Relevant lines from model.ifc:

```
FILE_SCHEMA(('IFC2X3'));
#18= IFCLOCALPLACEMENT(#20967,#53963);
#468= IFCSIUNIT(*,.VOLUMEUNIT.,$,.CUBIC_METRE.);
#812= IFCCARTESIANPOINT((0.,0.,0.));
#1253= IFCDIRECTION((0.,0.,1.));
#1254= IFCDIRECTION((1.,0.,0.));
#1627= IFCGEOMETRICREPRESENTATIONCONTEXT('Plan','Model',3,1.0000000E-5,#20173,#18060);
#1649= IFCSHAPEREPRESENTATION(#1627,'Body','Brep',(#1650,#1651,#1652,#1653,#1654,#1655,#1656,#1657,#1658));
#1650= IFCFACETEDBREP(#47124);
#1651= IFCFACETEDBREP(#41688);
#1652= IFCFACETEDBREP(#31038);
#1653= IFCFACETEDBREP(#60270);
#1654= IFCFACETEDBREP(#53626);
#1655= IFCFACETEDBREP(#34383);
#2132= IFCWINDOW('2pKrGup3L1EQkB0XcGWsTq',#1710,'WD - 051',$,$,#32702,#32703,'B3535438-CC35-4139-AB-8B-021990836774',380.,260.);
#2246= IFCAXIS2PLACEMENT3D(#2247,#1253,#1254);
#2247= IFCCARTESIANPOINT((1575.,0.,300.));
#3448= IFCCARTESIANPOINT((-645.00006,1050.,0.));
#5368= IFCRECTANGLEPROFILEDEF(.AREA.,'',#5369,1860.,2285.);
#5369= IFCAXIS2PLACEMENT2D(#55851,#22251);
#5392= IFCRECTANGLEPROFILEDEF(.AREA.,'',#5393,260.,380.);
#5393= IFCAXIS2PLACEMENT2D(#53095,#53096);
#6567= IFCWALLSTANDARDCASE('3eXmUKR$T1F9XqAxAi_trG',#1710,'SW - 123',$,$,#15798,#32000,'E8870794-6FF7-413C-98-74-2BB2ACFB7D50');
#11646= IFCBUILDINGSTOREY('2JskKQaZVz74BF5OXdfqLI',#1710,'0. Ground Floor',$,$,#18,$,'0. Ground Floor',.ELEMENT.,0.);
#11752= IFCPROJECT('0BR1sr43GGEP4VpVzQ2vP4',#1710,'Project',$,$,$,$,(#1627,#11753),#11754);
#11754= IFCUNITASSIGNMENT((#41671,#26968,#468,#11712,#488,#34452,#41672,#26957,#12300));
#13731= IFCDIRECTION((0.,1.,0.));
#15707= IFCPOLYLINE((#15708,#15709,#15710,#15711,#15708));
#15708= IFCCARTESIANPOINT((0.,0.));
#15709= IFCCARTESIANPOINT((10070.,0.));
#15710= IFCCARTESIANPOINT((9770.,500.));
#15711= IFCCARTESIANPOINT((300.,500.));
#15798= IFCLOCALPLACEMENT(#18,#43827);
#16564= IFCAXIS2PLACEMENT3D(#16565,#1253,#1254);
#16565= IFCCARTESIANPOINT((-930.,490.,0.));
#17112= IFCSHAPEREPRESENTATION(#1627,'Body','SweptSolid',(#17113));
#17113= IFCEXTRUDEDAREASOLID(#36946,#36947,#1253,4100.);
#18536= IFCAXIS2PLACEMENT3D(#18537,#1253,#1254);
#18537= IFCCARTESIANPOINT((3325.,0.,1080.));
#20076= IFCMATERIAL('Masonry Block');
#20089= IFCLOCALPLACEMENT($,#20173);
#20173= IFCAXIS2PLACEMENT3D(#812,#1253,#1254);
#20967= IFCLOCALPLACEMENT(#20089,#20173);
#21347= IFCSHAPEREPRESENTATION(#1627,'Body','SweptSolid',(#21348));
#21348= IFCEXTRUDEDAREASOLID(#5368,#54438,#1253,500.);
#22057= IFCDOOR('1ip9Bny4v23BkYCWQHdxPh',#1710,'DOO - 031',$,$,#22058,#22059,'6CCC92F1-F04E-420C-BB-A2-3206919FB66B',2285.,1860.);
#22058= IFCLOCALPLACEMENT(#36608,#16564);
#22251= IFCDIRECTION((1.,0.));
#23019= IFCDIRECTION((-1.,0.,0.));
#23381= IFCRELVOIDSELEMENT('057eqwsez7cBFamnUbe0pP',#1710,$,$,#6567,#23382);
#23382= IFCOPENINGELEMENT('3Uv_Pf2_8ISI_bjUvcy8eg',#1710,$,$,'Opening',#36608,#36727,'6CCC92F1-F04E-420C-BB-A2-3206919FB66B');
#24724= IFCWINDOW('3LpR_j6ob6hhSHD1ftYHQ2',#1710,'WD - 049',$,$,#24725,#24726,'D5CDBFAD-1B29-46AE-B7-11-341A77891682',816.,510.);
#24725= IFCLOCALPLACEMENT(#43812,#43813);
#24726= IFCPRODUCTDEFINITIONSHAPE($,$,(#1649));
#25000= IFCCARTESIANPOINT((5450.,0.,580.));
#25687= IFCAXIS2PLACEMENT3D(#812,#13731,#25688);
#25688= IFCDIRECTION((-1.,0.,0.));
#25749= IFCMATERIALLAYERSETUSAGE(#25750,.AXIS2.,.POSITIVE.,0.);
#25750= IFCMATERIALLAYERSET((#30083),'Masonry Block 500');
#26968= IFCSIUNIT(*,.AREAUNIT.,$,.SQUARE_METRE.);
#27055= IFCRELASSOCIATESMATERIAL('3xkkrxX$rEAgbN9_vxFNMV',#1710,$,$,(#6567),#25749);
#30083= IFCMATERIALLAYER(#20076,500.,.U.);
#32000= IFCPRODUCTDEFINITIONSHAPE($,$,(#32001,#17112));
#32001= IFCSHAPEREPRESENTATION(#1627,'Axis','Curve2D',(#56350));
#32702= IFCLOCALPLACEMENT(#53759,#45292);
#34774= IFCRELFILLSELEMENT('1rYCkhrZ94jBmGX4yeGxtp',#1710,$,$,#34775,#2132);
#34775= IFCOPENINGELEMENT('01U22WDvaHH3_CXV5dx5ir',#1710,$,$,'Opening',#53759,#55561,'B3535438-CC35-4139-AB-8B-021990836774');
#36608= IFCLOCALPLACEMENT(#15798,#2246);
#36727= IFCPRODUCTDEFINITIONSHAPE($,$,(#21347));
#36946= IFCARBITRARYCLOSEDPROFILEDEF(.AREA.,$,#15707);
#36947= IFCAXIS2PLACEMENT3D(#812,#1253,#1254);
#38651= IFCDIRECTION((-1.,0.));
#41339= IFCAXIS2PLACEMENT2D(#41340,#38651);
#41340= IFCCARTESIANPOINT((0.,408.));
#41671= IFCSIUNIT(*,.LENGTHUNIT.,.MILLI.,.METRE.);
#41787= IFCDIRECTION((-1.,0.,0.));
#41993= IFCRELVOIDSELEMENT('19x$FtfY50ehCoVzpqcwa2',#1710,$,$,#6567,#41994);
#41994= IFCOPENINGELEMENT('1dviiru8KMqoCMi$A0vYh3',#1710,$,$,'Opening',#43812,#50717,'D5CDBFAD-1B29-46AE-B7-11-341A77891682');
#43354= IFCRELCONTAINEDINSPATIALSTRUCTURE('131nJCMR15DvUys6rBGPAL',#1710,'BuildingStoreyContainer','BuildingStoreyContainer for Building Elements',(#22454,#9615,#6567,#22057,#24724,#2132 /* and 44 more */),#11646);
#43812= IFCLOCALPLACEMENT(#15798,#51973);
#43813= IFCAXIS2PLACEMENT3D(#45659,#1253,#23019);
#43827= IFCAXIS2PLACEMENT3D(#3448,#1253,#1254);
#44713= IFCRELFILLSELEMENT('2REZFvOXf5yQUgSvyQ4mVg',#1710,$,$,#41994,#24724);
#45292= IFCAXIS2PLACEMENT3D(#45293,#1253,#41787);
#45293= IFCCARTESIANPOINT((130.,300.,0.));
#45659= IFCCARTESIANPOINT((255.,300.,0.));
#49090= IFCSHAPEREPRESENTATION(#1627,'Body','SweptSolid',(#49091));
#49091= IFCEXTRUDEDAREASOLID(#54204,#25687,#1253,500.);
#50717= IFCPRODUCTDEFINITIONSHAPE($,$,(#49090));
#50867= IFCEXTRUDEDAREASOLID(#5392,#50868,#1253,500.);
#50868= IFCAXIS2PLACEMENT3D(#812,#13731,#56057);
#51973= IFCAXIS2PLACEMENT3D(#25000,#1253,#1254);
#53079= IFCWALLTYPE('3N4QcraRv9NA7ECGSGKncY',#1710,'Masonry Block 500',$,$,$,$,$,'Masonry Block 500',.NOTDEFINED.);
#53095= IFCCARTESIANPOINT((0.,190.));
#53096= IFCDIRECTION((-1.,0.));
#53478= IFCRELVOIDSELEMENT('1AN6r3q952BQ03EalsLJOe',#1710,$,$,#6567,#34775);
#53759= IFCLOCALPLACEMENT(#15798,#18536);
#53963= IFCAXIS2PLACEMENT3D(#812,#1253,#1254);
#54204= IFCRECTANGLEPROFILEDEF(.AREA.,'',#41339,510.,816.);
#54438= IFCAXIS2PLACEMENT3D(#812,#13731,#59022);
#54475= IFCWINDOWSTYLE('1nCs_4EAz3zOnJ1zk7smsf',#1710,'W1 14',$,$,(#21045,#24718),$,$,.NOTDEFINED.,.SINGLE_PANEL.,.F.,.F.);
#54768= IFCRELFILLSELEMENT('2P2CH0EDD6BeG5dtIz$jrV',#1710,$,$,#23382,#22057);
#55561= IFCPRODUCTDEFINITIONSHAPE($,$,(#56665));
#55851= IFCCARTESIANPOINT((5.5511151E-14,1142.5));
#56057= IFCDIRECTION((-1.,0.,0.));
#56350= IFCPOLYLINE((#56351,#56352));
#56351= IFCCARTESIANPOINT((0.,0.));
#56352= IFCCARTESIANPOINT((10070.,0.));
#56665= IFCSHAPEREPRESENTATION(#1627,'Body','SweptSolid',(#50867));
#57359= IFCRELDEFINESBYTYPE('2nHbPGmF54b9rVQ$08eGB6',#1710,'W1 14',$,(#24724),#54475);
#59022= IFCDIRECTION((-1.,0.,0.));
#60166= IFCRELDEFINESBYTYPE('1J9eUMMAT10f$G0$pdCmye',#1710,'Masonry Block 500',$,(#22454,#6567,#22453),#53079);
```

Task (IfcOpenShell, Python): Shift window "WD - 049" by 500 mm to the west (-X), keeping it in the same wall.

```python
import ifcopenshell
import ifcopenshell.api.geometry
import ifcopenshell.util.placement

model = ifcopenshell.open("model.ifc")

window = model.by_guid("3LpR_j6ob6hhSHD1ftYHQ2")
opening = window.FillsVoids[0].RelatingOpeningElement
wall = opening.VoidsElements[0].RelatingBuildingElement

wall_matrix = ifcopenshell.util.placement.get_local_placement(wall.ObjectPlacement)
shift = wall_matrix[:3, 0] * -500.0
before = ifcopenshell.util.placement.get_local_placement(window.ObjectPlacement)[:3, 3].copy()

# The window is placed relative to its opening, so it follows when the opening moves.
matrix = ifcopenshell.util.placement.get_local_placement(opening.ObjectPlacement)
matrix[:3, 3] += shift
ifcopenshell.api.geometry.edit_object_placement(
    model, product=opening, matrix=matrix, is_si=False, should_transform_children=True
)

after = ifcopenshell.util.placement.get_local_placement(window.ObjectPlacement)[:3, 3]
print("window moved by", (after - before).round(3) + 0.0)

model.write("model_v2.ifc")
```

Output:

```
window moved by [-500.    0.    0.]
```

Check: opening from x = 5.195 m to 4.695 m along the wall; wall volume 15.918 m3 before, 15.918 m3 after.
